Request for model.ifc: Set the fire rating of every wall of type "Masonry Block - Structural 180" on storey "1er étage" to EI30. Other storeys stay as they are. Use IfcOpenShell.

First a look at what the model holds.

```python
import ifcopenshell
import ifcopenshell.util.element

model = ifcopenshell.open("model.ifc")
print(model.schema)
storey = next(s for s in model.by_type("IfcBuildingStorey") if s.Name == "1er étage")
walls = [e for e in ifcopenshell.util.element.get_decomposition(storey) if e.is_a("IfcWall")]
seen = {}
for e in walls:
    element_type = ifcopenshell.util.element.get_type(e)
    key = (element_type.Name if element_type != e and element_type else None, ifcopenshell.util.element.get_pset(e, "Pset_WallCommon", "FireRating"))
    seen[key] = seen.get(key, 0) + 1
for (name, value), count in sorted(seen.items(), key=str):
    print(count, "x", name, "|", value)
```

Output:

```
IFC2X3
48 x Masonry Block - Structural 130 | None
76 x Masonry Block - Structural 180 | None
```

```python
import ifcopenshell
import ifcopenshell.api.pset
import ifcopenshell.util.element

model = ifcopenshell.open("model.ifc")

storey = next(s for s in model.by_type("IfcBuildingStorey") if s.Name == "1er étage")
walls = [e for e in ifcopenshell.util.element.get_decomposition(storey) if e.is_a("IfcWall")]

count = 0
for e in walls:
    element_type = ifcopenshell.util.element.get_type(e)
    if element_type in (None, e) or element_type.Name != "Masonry Block - Structural 180":
        continue
    # add_pset returns the element's existing set when there is one.
    pset = ifcopenshell.api.pset.add_pset(model, product=e, name="Pset_WallCommon")
    ifcopenshell.api.pset.edit_pset(model, pset=pset, properties={"FireRating": "EI30"})
    count += 1

print(count, "walls updated")

model.write("model_rev.ifc")
```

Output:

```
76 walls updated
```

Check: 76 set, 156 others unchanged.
